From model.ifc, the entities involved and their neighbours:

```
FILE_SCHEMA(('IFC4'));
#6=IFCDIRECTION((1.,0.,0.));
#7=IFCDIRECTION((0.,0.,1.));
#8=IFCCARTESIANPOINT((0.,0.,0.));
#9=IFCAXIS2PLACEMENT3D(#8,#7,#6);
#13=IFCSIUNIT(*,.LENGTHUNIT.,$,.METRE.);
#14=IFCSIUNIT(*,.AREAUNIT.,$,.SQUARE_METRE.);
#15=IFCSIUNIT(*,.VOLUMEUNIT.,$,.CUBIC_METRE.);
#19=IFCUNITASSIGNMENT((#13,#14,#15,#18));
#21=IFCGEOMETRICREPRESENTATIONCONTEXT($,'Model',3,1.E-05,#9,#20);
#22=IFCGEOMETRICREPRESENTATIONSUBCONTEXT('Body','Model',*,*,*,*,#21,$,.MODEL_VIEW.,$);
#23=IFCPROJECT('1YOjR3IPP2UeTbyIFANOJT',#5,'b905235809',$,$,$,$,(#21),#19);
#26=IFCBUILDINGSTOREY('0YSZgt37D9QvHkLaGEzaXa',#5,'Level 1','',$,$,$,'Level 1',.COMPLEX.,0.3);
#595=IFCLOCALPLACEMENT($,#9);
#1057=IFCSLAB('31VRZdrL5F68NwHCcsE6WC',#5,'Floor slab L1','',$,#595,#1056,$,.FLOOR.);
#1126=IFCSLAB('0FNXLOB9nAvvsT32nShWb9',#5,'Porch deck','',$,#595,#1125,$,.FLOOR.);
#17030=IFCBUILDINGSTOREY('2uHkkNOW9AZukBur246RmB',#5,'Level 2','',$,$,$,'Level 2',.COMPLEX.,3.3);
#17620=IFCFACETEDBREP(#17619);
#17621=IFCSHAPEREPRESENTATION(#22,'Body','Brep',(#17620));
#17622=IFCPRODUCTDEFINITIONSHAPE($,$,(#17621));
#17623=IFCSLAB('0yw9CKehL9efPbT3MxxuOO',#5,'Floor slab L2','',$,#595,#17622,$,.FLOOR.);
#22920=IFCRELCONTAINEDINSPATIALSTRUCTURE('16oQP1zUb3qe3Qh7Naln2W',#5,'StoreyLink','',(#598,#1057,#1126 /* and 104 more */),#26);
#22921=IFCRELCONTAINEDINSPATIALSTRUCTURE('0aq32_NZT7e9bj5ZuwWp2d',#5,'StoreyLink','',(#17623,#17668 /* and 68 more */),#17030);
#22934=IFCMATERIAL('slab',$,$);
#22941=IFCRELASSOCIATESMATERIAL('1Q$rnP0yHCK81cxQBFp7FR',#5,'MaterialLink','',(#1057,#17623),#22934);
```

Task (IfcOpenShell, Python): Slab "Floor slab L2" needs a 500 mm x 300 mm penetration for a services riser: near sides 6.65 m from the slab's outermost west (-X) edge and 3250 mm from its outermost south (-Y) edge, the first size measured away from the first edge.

```python
import numpy as np
import ifcopenshell
import ifcopenshell.api.feature
import ifcopenshell.api.geometry
import ifcopenshell.api.root
import ifcopenshell.geom
import ifcopenshell.util.placement
import ifcopenshell.util.representation
import ifcopenshell.util.shape
import ifcopenshell.util.unit

model = ifcopenshell.open("model.ifc")
unit_scale = ifcopenshell.util.unit.calculate_unit_scale(model)
settings = ifcopenshell.geom.settings()


def volume(element):
    """Net volume in cubic metres, openings subtracted."""
    shape = ifcopenshell.geom.create_shape(settings, element)
    return ifcopenshell.util.shape.get_volume(shape.geometry)


slab = model.by_guid("0yw9CKehL9efPbT3MxxuOO")
before = volume(slab)

# Extent in the slab's own axes, in metres. The edges named are its -X and -Y sides.
slab_shape = ifcopenshell.geom.create_shape(settings, slab)
vertices = ifcopenshell.util.shape.get_vertices(slab_shape.geometry)
x_min, y_min, bottom = vertices.min(axis=0)
top = vertices[:, 2].max()

opening = ifcopenshell.api.root.create_entity(model, ifc_class="IfcOpeningElement", name="Services riser opening", predefined_type="OPENING")
context = ifcopenshell.util.representation.get_context(model, "Model", "Body", "MODEL_VIEW")
width, depth = 0.5, 0.3
outline = [(0.0, 0.0), (width, 0.0), (width, depth), (0.0, depth), (0.0, 0.0)]
# Overshoot both faces by 50 mm so the cut is clean.
shape = ifcopenshell.api.geometry.add_slab_representation(
    model, context=context, depth=top - bottom + 0.1, polyline=outline
)
ifcopenshell.api.geometry.assign_representation(model, product=opening, representation=shape)

matrix = ifcopenshell.util.placement.get_local_placement(slab.ObjectPlacement)
matrix[:, 3] = matrix @ np.append(np.array([x_min + 6.65, y_min + 3.25, bottom - 0.05]) / unit_scale, 1.0)
ifcopenshell.api.geometry.edit_object_placement(model, product=opening, matrix=matrix, is_si=False)
ifcopenshell.api.feature.add_feature(model, feature=opening, element=slab)

after = volume(slab)

print(f"slab volume {before:.3f} -> {after:.3f} m3")

model.write("model_v2.ifc")
```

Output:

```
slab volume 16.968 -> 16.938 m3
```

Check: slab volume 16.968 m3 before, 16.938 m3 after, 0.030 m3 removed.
